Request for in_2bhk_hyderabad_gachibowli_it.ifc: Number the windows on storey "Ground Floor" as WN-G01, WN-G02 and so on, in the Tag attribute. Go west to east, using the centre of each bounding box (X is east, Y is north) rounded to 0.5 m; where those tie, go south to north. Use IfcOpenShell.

First a look at what the model holds.

```python
import ifcopenshell
import ifcopenshell.util.element
import ifcopenshell.util.placement

model = ifcopenshell.open("in_2bhk_hyderabad_gachibowli_it.ifc")
print(model.schema)
storey = next(s for s in model.by_type("IfcBuildingStorey") if s.Name == "Ground Floor")
windows = [e for e in ifcopenshell.util.element.get_decomposition(storey) if e.is_a("IfcWindow")]
for e in sorted(windows, key=lambda e: e.id()):
    origin = ifcopenshell.util.placement.get_local_placement(e.ObjectPlacement)[:3, 3]
    print(e.id(), e.Tag, e.Name, origin.round(2) + 0.0, sep=" | ")
```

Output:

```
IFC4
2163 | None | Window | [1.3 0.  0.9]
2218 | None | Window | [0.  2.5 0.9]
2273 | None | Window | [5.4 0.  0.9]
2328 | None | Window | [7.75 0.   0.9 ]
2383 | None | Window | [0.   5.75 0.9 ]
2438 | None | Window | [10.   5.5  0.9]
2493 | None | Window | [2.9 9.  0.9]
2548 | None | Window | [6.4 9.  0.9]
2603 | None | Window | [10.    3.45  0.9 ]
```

```python
import ifcopenshell
import ifcopenshell.geom
import ifcopenshell.util.element
import ifcopenshell.util.shape

model = ifcopenshell.open("in_2bhk_hyderabad_gachibowli_it.ifc")
settings = ifcopenshell.geom.settings()
settings.set("use-world-coords", True)


def centre(element):
    shape = ifcopenshell.geom.create_shape(settings, element)
    return ifcopenshell.util.shape.get_bbox_centroid(shape.geometry)


storey = next(s for s in model.by_type("IfcBuildingStorey") if s.Name == "Ground Floor")
windows = [e for e in ifcopenshell.util.element.get_decomposition(storey) if e.is_a("IfcWindow")]

# Insertion points can sit at a corner or the storey origin, so sort by the geometry (in metres).
centres = {e: centre(e) for e in windows}
windows.sort(key=lambda e: (round(centres[e][0] / 0.5), centres[e][1]))

for i, e in enumerate(windows, start=1):
    number = f"WN-G{i:02d}"
    e.Tag = number
    print(e.id(), number)

model.write("in_2bhk_hyderabad_gachibowli_it-out.ifc")
```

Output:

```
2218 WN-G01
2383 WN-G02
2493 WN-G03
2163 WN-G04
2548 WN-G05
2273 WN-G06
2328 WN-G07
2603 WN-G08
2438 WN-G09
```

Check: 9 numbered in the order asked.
